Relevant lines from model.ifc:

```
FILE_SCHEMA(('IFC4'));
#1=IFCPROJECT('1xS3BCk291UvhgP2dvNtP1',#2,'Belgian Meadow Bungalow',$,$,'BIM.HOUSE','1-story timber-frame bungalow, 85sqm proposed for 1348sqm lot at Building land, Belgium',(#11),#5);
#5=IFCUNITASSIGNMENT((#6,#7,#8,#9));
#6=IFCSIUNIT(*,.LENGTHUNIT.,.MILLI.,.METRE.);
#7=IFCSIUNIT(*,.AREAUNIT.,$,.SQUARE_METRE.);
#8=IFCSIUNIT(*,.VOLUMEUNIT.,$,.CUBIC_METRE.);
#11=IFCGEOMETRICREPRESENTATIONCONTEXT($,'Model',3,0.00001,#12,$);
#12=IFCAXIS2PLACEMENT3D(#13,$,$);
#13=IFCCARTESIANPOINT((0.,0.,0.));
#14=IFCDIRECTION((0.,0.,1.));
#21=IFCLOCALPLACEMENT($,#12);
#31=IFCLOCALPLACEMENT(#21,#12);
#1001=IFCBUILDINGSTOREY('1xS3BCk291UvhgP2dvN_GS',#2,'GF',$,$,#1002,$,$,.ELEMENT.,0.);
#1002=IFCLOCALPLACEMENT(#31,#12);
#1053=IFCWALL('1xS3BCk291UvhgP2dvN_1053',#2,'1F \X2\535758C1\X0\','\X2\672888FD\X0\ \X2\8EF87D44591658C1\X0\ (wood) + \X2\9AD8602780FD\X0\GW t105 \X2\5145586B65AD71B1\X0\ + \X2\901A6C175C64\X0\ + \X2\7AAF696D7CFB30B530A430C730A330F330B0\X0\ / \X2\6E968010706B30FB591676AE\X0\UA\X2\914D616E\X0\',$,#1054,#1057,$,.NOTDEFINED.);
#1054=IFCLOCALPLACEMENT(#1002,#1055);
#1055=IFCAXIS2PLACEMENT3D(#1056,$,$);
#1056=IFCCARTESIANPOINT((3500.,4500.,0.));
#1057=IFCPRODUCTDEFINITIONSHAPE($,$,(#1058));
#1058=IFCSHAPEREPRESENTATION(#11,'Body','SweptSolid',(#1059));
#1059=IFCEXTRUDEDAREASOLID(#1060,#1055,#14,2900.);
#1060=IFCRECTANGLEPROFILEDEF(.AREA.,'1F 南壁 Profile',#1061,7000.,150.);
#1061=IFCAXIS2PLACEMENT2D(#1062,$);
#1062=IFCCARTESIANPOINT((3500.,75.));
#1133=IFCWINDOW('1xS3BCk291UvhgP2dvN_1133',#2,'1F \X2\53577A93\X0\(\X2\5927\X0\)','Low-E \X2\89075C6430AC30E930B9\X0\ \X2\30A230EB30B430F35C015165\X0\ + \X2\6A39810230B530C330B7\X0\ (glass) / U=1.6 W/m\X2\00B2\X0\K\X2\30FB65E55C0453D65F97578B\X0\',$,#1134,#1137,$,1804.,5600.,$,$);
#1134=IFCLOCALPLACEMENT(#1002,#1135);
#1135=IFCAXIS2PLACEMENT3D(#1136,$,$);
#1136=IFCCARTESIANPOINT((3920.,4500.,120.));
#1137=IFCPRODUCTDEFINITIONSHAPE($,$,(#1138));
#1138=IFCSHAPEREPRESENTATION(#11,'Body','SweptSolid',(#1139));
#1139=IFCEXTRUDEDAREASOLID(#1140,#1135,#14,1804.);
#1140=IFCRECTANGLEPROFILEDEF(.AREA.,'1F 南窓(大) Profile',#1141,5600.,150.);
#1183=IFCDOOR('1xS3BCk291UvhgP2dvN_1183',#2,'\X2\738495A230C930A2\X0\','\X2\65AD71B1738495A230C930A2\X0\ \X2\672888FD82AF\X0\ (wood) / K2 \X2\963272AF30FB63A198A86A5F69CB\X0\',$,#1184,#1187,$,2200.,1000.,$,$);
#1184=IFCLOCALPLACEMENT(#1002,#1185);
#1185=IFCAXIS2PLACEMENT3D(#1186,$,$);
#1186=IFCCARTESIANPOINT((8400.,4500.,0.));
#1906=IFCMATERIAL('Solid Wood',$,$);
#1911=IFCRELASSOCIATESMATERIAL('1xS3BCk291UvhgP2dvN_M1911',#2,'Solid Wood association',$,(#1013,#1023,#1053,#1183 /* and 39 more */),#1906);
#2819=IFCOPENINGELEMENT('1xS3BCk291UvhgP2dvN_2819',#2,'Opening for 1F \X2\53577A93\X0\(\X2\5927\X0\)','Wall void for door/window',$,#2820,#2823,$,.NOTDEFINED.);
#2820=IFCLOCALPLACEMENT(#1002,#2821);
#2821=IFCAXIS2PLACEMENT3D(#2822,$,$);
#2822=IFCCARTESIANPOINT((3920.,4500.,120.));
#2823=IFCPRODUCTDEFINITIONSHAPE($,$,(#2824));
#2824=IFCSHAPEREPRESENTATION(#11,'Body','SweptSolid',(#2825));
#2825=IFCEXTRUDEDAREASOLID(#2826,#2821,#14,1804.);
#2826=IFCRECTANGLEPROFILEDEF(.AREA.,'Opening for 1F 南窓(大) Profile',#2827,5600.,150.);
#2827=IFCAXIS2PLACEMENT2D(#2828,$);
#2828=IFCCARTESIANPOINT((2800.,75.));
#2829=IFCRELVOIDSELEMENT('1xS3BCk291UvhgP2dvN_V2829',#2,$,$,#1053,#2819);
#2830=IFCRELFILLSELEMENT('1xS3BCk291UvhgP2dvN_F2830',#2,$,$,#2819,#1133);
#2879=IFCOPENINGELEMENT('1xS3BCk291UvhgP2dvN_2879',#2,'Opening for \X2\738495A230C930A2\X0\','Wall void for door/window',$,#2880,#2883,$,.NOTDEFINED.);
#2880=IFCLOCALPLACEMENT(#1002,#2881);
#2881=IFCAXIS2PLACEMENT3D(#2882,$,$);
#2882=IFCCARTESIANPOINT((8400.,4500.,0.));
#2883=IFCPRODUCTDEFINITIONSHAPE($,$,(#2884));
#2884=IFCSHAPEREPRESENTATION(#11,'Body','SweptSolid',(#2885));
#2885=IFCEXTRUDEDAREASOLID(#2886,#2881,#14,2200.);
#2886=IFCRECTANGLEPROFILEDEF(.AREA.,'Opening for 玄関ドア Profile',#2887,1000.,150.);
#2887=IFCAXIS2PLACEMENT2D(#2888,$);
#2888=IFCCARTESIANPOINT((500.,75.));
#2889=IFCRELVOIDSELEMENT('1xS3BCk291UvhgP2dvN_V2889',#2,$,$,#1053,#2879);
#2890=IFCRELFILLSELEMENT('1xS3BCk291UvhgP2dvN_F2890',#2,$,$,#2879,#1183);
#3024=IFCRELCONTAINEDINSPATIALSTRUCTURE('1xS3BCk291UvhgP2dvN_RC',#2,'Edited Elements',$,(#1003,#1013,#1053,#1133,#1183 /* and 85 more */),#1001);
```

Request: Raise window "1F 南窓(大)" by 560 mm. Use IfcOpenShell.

```python
import numpy as np
import ifcopenshell
import ifcopenshell.api.geometry
import ifcopenshell.util.placement
import ifcopenshell.util.unit

model = ifcopenshell.open("model.ifc")
unit_scale = ifcopenshell.util.unit.calculate_unit_scale(model)

window = model.by_guid("1xS3BCk291UvhgP2dvN_1133")
opening = window.FillsVoids[0].RelatingOpeningElement
dz = 560.0

shift = np.array([0.0, 0.0, dz])
# The window is not placed relative to its opening, so move both.
for product in (opening, window):
    matrix = ifcopenshell.util.placement.get_local_placement(product.ObjectPlacement)
    matrix[:3, 3] += shift
    ifcopenshell.api.geometry.edit_object_placement(model, product=product, matrix=matrix, is_si=False)

print(f"moved by {dz * unit_scale:+.3f} m")

model.write("model_updated.ifc")
```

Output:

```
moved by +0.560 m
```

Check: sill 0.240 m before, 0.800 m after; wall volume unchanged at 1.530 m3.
